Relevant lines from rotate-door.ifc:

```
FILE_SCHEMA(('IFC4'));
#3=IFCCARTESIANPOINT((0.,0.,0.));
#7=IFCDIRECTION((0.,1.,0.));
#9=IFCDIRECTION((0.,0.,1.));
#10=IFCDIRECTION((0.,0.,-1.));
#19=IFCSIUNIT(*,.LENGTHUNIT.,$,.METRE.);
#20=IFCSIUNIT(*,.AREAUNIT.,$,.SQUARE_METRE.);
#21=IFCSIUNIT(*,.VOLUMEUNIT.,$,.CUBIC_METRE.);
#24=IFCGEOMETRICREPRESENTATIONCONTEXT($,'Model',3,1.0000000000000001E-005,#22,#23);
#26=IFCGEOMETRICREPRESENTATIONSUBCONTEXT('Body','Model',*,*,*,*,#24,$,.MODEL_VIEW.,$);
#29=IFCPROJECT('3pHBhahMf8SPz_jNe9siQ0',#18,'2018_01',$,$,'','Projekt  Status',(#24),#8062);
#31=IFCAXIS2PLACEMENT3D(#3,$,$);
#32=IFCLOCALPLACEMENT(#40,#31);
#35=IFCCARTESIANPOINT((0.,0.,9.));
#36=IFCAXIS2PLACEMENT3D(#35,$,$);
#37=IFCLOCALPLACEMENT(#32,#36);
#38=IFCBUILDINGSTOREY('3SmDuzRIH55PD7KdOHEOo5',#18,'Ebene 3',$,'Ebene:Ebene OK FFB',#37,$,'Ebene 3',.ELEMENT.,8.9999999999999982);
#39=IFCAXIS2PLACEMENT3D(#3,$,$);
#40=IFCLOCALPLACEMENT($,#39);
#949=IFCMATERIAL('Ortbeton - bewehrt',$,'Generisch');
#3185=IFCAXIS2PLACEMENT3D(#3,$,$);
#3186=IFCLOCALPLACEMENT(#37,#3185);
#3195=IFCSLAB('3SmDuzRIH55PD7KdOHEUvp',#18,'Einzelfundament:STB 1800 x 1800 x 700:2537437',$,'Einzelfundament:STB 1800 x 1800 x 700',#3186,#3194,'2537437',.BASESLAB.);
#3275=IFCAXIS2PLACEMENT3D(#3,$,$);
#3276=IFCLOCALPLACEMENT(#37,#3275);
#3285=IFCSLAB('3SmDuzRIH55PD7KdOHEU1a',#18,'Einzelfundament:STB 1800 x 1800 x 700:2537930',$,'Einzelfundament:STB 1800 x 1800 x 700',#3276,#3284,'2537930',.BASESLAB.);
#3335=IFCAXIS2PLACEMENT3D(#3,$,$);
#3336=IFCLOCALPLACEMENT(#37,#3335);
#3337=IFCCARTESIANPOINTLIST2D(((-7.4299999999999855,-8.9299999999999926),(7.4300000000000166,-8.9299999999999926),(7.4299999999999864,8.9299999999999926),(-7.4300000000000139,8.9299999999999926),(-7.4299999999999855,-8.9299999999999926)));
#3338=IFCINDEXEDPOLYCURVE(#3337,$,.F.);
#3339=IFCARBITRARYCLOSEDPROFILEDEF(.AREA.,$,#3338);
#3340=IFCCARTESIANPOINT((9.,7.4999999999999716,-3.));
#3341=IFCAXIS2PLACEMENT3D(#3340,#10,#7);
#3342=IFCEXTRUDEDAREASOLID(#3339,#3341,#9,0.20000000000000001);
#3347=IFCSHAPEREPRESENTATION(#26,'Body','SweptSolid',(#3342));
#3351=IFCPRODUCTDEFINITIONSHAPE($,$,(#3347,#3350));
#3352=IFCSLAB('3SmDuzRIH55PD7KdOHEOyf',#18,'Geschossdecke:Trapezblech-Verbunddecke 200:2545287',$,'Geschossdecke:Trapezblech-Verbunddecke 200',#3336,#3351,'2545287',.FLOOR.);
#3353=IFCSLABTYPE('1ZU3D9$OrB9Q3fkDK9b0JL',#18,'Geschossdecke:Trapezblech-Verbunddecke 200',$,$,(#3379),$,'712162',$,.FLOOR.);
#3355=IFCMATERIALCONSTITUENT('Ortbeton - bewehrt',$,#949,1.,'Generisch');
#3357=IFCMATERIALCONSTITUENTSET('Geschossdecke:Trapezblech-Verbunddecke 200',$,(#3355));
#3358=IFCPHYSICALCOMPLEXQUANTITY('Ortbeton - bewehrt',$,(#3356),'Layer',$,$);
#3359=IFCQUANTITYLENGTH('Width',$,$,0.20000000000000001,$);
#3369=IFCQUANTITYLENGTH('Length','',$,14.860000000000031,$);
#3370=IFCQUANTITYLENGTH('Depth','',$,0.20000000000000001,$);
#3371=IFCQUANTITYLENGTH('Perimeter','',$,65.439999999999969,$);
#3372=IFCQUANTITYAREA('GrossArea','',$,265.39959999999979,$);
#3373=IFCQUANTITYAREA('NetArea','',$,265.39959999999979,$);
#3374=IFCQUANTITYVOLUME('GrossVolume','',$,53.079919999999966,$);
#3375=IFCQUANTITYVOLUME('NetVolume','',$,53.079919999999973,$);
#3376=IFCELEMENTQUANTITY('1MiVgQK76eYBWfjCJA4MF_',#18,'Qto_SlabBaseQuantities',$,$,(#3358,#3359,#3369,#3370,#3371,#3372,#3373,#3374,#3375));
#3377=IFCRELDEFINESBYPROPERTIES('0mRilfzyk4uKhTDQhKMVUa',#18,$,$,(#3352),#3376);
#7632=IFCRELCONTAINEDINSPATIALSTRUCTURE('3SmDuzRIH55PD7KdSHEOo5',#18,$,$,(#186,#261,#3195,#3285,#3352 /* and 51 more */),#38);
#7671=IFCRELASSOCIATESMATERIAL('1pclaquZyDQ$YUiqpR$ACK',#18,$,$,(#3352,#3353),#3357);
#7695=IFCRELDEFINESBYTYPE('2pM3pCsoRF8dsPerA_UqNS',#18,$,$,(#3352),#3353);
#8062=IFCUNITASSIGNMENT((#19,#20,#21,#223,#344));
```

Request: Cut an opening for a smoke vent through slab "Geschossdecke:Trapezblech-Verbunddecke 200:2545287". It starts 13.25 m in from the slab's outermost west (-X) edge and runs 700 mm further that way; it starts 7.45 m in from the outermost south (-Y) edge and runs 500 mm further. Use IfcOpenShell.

```python
import numpy as np
import ifcopenshell
import ifcopenshell.api.feature
import ifcopenshell.api.geometry
import ifcopenshell.api.pset
import ifcopenshell.api.root
import ifcopenshell.geom
import ifcopenshell.util.element
import ifcopenshell.util.placement
import ifcopenshell.util.representation
import ifcopenshell.util.shape
import ifcopenshell.util.unit

model = ifcopenshell.open("rotate-door.ifc")
unit_scale = ifcopenshell.util.unit.calculate_unit_scale(model)
area_scale = ifcopenshell.util.unit.calculate_unit_scale(model, "AREAUNIT")
volume_scale = ifcopenshell.util.unit.calculate_unit_scale(model, "VOLUMEUNIT")
settings = ifcopenshell.geom.settings()


def volume(element):
    """Net volume in cubic metres, openings subtracted."""
    shape = ifcopenshell.geom.create_shape(settings, element)
    return ifcopenshell.util.shape.get_volume(shape.geometry)


slab = model.by_id(3352)
before = volume(slab)

# Extent in the slab's own axes, in metres. The edges named are its -X and -Y sides.
slab_shape = ifcopenshell.geom.create_shape(settings, slab)
vertices = ifcopenshell.util.shape.get_vertices(slab_shape.geometry)
x_min, y_min, bottom = vertices.min(axis=0)
top = vertices[:, 2].max()

opening = ifcopenshell.api.root.create_entity(model, ifc_class="IfcOpeningElement", name="Smoke vent opening", predefined_type="OPENING")
context = ifcopenshell.util.representation.get_context(model, "Model", "Body", "MODEL_VIEW")
width, depth = 0.7, 0.5
outline = [(0.0, 0.0), (width, 0.0), (width, depth), (0.0, depth), (0.0, 0.0)]
# Overshoot both faces by 50 mm so the cut is clean.
shape = ifcopenshell.api.geometry.add_slab_representation(
    model, context=context, depth=top - bottom + 0.1, polyline=outline
)
ifcopenshell.api.geometry.assign_representation(model, product=opening, representation=shape)

matrix = ifcopenshell.util.placement.get_local_placement(slab.ObjectPlacement)
matrix[:, 3] = matrix @ np.append(np.array([x_min + 13.25, y_min + 7.45, bottom - 0.05]) / unit_scale, 1.0)
ifcopenshell.api.geometry.edit_object_placement(model, product=opening, matrix=matrix, is_si=False)
ifcopenshell.api.feature.add_feature(model, feature=opening, element=slab)

after = volume(slab)

# Update the slab's stored quantities.
qto = model.by_id(ifcopenshell.util.element.get_pset(slab, "Qto_SlabBaseQuantities", should_inherit=False)["id"])
ifcopenshell.api.pset.edit_qto(model, qto=qto, properties={
    "NetArea": after / (top - bottom) / area_scale,
    "NetVolume": after / volume_scale,
})

print(f"slab volume {before:.3f} -> {after:.3f} m3")

model.write("rotate-door-out.ifc")
```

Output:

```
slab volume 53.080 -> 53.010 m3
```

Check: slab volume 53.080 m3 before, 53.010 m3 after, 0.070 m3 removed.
